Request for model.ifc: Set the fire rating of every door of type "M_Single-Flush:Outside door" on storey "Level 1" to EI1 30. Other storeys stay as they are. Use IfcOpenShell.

First a look at what the model holds.

```python
import ifcopenshell
import ifcopenshell.util.element

model = ifcopenshell.open("model.ifc")
print(model.schema)
storey = next(s for s in model.by_type("IfcBuildingStorey") if s.Name == "Level 1")
doors = [e for e in ifcopenshell.util.element.get_decomposition(storey) if e.is_a("IfcDoor")]
seen = {}
for e in doors:
    element_type = ifcopenshell.util.element.get_type(e)
    key = (element_type.Name if element_type != e and element_type else None, ifcopenshell.util.element.get_pset(e, "Pset_DoorCommon", "FireRating"))
    seen[key] = seen.get(key, 0) + 1
for (name, value), count in sorted(seen.items(), key=str):
    print(count, "x", name, "|", value)
```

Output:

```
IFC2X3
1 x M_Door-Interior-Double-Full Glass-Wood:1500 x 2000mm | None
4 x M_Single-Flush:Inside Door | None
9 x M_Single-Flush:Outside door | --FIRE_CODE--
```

```python
import ifcopenshell
import ifcopenshell.api.pset
import ifcopenshell.util.element

model = ifcopenshell.open("model.ifc")

storey = next(s for s in model.by_type("IfcBuildingStorey") if s.Name == "Level 1")
doors = [e for e in ifcopenshell.util.element.get_decomposition(storey) if e.is_a("IfcDoor")]

count = 0
for e in doors:
    element_type = ifcopenshell.util.element.get_type(e)
    if element_type in (None, e) or element_type.Name != "M_Single-Flush:Outside door":
        continue
    # add_pset returns the element's existing set when there is one.
    pset = ifcopenshell.api.pset.add_pset(model, product=e, name="Pset_DoorCommon")
    ifcopenshell.api.pset.edit_pset(model, pset=pset, properties={"FireRating": "EI1 30"})
    count += 1

print(count, "doors updated")

model.write("model-out.ifc")
```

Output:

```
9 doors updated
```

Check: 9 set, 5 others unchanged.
